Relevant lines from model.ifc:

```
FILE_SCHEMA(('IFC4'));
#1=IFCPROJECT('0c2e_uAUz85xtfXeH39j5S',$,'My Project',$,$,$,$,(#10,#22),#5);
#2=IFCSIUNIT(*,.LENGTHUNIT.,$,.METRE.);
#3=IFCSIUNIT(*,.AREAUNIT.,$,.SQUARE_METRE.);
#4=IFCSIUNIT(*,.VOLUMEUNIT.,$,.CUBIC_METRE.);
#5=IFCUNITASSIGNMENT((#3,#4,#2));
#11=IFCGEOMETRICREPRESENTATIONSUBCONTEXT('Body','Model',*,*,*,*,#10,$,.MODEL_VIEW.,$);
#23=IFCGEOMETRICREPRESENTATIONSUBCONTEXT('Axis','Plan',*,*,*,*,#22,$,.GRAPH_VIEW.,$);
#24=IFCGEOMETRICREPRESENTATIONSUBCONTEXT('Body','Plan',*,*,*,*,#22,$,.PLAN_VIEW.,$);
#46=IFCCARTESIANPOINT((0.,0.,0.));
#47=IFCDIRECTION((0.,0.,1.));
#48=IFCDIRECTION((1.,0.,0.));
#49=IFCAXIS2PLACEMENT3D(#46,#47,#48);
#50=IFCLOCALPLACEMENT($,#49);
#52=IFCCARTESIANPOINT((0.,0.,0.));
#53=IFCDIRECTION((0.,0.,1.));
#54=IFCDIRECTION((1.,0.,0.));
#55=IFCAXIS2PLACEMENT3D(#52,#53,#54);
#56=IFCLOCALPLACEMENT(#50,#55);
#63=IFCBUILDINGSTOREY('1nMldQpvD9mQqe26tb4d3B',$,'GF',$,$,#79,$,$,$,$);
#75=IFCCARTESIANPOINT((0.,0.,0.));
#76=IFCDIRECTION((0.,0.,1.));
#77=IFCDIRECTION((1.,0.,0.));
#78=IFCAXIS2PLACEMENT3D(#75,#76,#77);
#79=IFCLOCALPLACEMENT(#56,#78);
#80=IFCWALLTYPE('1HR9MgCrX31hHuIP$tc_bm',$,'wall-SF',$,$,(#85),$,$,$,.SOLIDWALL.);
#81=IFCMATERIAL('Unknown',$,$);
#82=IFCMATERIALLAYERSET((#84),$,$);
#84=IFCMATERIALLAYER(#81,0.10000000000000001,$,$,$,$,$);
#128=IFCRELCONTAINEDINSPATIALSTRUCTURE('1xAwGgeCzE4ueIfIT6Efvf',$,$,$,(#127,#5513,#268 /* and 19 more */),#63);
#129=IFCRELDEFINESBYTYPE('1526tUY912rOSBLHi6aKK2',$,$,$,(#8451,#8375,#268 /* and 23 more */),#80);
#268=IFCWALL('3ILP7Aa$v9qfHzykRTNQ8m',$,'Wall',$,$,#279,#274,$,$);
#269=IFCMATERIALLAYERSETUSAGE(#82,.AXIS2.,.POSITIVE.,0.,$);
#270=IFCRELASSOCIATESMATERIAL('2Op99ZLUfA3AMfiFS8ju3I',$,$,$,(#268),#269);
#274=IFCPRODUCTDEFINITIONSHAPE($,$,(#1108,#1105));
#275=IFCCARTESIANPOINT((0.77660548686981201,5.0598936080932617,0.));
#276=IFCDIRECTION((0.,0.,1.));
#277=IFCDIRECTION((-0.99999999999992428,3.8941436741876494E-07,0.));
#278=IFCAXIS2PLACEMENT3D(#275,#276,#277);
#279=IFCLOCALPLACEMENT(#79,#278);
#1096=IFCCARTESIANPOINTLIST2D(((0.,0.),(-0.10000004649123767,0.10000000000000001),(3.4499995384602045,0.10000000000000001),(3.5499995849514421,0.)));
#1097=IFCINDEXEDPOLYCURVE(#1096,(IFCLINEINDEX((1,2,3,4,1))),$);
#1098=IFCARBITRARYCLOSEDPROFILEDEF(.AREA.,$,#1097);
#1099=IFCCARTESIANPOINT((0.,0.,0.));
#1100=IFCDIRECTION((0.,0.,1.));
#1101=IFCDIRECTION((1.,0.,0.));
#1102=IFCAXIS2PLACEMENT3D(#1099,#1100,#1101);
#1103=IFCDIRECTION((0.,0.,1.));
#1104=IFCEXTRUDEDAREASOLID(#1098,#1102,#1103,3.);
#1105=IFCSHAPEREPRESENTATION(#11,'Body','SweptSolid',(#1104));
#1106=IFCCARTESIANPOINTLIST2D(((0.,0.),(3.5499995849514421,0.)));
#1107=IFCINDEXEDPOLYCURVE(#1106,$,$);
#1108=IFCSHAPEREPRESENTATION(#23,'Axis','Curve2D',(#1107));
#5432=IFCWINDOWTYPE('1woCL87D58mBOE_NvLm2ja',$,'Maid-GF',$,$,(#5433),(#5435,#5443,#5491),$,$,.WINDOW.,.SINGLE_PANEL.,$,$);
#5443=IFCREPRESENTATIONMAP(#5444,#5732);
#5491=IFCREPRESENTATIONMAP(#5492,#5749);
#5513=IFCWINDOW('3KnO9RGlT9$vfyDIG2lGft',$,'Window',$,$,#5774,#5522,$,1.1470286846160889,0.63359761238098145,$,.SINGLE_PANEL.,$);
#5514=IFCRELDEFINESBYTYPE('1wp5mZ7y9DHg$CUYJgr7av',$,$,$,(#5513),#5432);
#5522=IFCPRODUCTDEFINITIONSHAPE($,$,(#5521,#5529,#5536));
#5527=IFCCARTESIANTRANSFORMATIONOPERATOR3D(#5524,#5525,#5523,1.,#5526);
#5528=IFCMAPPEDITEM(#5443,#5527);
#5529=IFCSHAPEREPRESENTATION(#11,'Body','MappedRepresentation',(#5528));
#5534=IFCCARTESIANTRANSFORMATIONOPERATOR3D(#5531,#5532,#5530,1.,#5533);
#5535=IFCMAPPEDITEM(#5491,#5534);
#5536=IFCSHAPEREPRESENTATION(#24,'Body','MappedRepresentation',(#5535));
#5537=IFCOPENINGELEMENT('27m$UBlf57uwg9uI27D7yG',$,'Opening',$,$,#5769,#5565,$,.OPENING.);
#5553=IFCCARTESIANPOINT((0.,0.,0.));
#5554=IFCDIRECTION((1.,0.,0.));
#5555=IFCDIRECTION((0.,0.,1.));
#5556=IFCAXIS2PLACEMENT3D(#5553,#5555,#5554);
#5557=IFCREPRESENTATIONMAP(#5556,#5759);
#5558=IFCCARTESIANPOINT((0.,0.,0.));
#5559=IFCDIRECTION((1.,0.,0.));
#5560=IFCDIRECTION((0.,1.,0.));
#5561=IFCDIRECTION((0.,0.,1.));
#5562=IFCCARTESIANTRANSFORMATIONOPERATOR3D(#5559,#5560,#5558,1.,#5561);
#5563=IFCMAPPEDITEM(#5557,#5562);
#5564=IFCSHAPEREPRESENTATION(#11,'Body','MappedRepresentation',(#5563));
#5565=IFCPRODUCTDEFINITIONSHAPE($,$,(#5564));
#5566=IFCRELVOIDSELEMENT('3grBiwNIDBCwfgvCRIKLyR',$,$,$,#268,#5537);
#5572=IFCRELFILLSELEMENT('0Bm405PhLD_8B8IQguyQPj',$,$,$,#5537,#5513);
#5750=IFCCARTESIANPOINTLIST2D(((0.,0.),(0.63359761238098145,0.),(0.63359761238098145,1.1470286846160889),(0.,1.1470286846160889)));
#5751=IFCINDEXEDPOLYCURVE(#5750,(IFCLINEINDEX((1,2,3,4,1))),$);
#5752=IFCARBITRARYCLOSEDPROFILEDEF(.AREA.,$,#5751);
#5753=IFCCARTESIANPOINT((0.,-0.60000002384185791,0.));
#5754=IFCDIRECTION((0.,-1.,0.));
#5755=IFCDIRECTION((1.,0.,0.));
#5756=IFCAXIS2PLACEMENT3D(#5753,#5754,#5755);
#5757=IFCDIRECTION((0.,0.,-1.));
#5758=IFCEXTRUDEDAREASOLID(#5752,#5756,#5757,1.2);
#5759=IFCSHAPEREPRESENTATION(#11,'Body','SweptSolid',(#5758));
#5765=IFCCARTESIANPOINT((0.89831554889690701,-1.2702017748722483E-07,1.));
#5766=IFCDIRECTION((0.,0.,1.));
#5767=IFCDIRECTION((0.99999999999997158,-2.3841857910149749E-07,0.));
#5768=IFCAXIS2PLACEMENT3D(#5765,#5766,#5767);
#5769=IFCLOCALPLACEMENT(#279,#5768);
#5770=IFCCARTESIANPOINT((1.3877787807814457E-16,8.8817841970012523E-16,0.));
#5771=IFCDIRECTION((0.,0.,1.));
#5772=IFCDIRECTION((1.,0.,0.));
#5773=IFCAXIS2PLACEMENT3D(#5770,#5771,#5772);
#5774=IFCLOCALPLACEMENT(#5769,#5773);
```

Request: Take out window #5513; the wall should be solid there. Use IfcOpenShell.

```python
import ifcopenshell
import ifcopenshell.api.feature
import ifcopenshell.api.root
import ifcopenshell.geom
import ifcopenshell.util.shape

model = ifcopenshell.open("model.ifc")
settings = ifcopenshell.geom.settings()


def volume(element):
    """Net volume in cubic metres, openings subtracted."""
    shape = ifcopenshell.geom.create_shape(settings, element)
    return ifcopenshell.util.shape.get_volume(shape.geometry)


window = model.by_id(5513)
opening = window.FillsVoids[0].RelatingOpeningElement
wall = opening.VoidsElements[0].RelatingBuildingElement
before = volume(wall)

ifcopenshell.api.root.remove_product(model, product=window)
ifcopenshell.api.feature.remove_feature(model, feature=opening)

after = volume(wall)

print(f"wall volume {before:.3f} -> {after:.3f} m3")

model.write("model_updated.ifc")
```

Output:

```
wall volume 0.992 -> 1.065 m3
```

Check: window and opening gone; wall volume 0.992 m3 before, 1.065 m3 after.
